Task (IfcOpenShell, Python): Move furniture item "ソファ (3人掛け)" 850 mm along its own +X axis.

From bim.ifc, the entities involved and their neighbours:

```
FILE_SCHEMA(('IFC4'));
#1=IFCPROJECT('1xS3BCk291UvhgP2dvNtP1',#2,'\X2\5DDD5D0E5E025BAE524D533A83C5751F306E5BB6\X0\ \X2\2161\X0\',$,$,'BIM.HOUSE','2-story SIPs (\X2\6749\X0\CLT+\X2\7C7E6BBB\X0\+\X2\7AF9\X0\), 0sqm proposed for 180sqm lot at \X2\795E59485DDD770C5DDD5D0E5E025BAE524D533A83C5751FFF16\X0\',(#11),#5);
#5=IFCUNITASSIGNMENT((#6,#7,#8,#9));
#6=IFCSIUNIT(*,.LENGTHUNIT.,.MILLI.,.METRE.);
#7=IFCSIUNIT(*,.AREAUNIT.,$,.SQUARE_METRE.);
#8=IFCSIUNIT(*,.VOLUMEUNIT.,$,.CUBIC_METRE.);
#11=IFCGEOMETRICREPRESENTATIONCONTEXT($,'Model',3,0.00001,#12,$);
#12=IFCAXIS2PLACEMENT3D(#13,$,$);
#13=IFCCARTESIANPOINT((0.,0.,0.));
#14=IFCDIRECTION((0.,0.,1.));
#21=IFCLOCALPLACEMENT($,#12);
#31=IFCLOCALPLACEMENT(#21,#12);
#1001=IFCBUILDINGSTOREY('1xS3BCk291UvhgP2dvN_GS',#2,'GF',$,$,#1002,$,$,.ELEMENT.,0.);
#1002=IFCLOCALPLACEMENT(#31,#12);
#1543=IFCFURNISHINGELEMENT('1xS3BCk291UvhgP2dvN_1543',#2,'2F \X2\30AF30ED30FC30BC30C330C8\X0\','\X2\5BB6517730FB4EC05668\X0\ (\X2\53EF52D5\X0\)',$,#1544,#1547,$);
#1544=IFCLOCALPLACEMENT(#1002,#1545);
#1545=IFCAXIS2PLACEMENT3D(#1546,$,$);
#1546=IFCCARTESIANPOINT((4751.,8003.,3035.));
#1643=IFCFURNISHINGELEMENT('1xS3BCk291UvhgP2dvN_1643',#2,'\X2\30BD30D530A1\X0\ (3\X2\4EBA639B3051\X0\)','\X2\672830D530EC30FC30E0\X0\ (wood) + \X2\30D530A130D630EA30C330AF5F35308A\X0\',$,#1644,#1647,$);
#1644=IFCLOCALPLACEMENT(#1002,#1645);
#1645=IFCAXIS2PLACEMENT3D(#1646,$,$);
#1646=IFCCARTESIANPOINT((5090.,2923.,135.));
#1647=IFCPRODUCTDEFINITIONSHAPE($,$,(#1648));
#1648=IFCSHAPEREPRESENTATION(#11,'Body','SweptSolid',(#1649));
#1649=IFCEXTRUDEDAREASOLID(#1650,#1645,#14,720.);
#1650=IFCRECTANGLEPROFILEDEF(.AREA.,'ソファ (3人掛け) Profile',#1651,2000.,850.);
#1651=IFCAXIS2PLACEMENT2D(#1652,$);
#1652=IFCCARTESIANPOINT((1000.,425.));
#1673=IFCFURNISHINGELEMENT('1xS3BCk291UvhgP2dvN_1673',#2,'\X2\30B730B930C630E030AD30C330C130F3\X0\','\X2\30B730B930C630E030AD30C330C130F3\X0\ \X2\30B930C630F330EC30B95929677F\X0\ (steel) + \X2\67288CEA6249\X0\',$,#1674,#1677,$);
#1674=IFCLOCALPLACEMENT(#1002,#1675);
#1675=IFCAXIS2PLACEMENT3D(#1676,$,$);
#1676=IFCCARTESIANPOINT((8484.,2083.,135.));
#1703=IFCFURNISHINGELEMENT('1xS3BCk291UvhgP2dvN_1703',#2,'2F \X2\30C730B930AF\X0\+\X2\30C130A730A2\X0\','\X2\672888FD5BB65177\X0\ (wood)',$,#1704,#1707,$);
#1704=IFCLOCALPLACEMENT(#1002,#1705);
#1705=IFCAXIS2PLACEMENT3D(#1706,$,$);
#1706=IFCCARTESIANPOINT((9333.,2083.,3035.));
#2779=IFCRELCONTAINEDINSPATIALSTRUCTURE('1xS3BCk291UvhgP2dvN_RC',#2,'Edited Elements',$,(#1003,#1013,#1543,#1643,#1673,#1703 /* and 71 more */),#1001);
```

```python
import ifcopenshell
import ifcopenshell.api.geometry
import ifcopenshell.util.placement
import ifcopenshell.util.unit

model = ifcopenshell.open("bim.ifc")
unit_scale = ifcopenshell.util.unit.calculate_unit_scale(model)

item = model.by_id(1643)
matrix = ifcopenshell.util.placement.get_local_placement(item.ObjectPlacement)
matrix[:3, 3] += matrix[:3, 0] * 0.85 / unit_scale
ifcopenshell.api.geometry.edit_object_placement(model, product=item, matrix=matrix, is_si=False)

print(ifcopenshell.util.placement.get_local_placement(item.ObjectPlacement).round(3) + 0.0)

model.write("bim_updated.ifc")
```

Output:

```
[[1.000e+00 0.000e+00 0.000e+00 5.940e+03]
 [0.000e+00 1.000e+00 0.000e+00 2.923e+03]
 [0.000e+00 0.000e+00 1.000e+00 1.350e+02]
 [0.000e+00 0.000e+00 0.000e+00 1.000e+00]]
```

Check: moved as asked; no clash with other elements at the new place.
